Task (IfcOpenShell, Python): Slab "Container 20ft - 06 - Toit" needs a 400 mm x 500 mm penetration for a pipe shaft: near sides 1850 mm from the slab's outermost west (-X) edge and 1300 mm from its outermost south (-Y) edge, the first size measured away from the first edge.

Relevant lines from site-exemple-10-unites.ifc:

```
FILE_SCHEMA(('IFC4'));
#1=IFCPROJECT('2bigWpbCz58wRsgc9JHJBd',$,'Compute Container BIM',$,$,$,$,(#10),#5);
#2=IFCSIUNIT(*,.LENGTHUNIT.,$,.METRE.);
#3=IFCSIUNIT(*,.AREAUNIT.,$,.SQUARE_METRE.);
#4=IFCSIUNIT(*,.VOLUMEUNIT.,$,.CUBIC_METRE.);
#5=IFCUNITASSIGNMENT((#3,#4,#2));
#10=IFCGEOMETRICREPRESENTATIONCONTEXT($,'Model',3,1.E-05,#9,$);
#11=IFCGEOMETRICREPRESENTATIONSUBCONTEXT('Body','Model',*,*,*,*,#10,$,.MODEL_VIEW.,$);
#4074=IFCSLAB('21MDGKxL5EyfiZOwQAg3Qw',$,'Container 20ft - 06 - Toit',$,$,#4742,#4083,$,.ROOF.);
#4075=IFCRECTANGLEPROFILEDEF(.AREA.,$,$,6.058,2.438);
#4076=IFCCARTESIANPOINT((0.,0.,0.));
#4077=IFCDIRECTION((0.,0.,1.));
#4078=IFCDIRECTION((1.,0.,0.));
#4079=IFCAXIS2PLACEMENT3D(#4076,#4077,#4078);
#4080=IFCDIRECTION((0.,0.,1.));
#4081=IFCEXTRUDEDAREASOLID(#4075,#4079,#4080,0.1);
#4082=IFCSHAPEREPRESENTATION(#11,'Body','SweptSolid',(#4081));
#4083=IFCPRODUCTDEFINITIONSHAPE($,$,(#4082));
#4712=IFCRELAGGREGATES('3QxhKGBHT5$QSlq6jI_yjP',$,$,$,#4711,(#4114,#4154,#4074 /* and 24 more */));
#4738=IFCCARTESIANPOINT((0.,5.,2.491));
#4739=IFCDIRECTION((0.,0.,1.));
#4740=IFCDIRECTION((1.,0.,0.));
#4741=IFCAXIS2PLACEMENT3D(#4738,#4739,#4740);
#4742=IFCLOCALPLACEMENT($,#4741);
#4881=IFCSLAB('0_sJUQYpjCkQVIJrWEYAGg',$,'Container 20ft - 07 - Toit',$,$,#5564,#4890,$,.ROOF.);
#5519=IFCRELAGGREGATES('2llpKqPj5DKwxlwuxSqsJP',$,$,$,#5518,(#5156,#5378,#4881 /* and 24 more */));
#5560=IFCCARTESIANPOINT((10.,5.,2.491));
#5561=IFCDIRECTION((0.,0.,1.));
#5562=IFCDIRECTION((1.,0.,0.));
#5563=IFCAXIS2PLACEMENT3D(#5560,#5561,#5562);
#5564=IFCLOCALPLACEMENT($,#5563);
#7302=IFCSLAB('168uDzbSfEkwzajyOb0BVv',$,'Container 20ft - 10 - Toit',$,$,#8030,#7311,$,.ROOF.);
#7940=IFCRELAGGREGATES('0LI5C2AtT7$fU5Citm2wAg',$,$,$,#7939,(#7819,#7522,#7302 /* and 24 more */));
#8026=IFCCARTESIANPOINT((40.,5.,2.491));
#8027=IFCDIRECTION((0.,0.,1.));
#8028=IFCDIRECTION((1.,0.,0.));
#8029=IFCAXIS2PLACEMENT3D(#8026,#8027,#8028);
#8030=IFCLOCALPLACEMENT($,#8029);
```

```python
import numpy as np
import ifcopenshell
import ifcopenshell.api.feature
import ifcopenshell.api.geometry
import ifcopenshell.api.root
import ifcopenshell.geom
import ifcopenshell.util.placement
import ifcopenshell.util.representation
import ifcopenshell.util.shape
import ifcopenshell.util.unit

model = ifcopenshell.open("site-exemple-10-unites.ifc")
unit_scale = ifcopenshell.util.unit.calculate_unit_scale(model)
settings = ifcopenshell.geom.settings()


def volume(element):
    """Net volume in cubic metres, openings subtracted."""
    shape = ifcopenshell.geom.create_shape(settings, element)
    return ifcopenshell.util.shape.get_volume(shape.geometry)


slab = model.by_guid("21MDGKxL5EyfiZOwQAg3Qw")
before = volume(slab)

# Extent in the slab's own axes, in metres. The edges named are its -X and -Y sides.
slab_shape = ifcopenshell.geom.create_shape(settings, slab)
vertices = ifcopenshell.util.shape.get_vertices(slab_shape.geometry)
x_min, y_min, bottom = vertices.min(axis=0)
top = vertices[:, 2].max()

opening = ifcopenshell.api.root.create_entity(model, ifc_class="IfcOpeningElement", name="Pipe shaft opening", predefined_type="OPENING")
context = ifcopenshell.util.representation.get_context(model, "Model", "Body", "MODEL_VIEW")
width, depth = 0.4, 0.5
outline = [(0.0, 0.0), (width, 0.0), (width, depth), (0.0, depth), (0.0, 0.0)]
# Overshoot both faces by 50 mm so the cut is clean.
shape = ifcopenshell.api.geometry.add_slab_representation(
    model, context=context, depth=top - bottom + 0.1, polyline=outline
)
ifcopenshell.api.geometry.assign_representation(model, product=opening, representation=shape)

matrix = ifcopenshell.util.placement.get_local_placement(slab.ObjectPlacement)
matrix[:, 3] = matrix @ np.append(np.array([x_min + 1.85, y_min + 1.3, bottom - 0.05]) / unit_scale, 1.0)
ifcopenshell.api.geometry.edit_object_placement(model, product=opening, matrix=matrix, is_si=False)
ifcopenshell.api.feature.add_feature(model, feature=opening, element=slab)

after = volume(slab)

print(f"slab volume {before:.3f} -> {after:.3f} m3")

model.write("site-exemple-10-unites-out.ifc")
```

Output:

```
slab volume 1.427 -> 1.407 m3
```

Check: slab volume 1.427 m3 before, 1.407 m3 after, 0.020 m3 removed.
